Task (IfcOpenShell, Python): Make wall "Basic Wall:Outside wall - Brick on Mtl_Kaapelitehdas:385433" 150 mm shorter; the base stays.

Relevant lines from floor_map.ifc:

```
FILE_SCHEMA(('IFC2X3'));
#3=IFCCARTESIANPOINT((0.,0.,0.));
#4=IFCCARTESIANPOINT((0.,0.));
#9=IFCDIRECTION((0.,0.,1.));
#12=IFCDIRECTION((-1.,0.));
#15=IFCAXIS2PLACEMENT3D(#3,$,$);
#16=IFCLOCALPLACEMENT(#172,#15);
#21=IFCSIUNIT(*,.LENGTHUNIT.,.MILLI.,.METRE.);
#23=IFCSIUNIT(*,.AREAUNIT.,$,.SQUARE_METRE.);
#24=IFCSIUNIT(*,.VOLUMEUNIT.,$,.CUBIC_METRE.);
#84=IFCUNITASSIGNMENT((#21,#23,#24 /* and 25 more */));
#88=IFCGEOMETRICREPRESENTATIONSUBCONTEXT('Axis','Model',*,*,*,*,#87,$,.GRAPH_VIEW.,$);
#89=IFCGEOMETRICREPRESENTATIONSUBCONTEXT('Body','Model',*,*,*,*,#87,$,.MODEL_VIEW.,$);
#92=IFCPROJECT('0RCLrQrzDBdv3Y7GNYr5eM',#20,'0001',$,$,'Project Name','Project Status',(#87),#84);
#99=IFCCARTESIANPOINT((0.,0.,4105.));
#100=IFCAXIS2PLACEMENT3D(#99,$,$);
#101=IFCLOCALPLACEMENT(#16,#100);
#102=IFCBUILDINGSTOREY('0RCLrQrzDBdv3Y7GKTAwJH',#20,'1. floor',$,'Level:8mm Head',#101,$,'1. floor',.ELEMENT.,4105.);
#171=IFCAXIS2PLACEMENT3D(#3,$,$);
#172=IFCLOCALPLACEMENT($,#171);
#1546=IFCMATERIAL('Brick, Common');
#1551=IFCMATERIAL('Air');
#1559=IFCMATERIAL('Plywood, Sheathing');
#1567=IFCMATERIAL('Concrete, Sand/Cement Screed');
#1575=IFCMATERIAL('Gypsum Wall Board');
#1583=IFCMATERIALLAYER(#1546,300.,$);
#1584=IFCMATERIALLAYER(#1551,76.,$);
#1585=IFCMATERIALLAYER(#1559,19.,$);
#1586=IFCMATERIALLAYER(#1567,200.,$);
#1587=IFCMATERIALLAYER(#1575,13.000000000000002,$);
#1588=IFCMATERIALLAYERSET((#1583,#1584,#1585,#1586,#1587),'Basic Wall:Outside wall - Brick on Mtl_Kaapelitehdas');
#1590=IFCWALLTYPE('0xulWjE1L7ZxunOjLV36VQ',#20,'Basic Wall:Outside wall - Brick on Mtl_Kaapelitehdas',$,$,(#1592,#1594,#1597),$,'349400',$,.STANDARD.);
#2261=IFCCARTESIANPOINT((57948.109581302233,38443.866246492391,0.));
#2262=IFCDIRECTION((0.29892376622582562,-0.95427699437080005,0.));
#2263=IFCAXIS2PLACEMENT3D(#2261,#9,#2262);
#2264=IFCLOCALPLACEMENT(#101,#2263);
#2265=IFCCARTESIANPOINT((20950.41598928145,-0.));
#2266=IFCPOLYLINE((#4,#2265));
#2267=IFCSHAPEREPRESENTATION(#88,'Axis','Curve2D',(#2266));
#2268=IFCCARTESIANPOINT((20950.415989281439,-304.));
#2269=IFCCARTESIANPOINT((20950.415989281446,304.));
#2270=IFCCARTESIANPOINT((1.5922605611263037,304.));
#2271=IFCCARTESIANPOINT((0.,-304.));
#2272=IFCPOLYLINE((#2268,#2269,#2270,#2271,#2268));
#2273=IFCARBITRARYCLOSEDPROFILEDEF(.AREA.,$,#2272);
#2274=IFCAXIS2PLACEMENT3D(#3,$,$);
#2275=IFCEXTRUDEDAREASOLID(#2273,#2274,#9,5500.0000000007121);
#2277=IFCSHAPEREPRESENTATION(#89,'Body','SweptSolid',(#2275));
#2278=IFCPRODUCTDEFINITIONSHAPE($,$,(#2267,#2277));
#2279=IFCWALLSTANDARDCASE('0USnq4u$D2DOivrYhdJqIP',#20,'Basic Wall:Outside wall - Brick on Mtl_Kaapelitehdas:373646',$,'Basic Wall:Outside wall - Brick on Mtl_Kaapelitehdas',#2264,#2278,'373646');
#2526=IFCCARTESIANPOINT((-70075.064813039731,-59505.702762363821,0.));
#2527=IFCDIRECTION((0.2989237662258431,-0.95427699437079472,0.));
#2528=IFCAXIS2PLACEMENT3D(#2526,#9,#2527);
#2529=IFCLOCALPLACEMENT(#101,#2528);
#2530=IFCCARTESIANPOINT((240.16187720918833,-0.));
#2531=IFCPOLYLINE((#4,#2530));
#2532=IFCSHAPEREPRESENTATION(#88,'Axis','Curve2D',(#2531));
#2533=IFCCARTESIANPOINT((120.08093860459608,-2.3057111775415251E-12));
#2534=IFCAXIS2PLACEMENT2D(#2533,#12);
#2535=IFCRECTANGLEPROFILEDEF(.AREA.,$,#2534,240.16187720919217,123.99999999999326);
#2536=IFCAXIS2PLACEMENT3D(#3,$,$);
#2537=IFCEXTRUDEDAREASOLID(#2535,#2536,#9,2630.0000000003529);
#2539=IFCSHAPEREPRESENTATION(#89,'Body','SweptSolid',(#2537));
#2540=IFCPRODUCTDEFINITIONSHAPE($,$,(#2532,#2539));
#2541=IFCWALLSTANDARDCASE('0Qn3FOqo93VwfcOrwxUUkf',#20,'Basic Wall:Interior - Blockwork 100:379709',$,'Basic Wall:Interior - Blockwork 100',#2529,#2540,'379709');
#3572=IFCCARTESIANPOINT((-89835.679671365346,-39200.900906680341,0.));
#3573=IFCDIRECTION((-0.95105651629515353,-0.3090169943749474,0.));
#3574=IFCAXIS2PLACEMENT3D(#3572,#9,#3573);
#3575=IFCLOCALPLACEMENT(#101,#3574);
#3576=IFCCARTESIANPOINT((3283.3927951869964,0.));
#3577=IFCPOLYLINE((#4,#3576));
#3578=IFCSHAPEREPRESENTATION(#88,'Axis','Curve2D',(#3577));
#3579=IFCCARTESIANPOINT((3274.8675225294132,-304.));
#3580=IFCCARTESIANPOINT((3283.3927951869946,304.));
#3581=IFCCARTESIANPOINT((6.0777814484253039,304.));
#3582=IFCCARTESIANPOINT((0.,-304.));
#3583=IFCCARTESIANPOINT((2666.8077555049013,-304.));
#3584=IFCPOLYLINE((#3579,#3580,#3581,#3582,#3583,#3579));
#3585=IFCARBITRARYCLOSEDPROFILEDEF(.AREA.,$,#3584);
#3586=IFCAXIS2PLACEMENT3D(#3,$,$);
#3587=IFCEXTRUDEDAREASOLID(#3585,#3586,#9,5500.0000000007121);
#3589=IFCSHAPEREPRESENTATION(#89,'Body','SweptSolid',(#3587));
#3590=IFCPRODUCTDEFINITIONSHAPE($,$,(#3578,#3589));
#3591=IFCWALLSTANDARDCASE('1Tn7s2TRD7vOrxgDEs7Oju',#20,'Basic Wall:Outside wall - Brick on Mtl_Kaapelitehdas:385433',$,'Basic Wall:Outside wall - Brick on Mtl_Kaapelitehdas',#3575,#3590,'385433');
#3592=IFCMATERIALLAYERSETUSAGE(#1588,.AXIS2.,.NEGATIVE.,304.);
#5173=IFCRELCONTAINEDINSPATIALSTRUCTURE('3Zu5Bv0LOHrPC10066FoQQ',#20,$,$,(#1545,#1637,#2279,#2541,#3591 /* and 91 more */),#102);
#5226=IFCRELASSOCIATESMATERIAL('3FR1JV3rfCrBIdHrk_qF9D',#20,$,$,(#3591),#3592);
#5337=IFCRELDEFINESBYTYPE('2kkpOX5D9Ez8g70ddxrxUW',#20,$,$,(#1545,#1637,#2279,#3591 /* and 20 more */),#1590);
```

```python
import ifcopenshell
import ifcopenshell.geom
import ifcopenshell.util.representation
import ifcopenshell.util.shape

model = ifcopenshell.open("floor_map.ifc")
settings = ifcopenshell.geom.settings()


def volume(element):
    """Net volume in cubic metres, openings subtracted."""
    shape = ifcopenshell.geom.create_shape(settings, element)
    return ifcopenshell.util.shape.get_volume(shape.geometry)


wall = model.by_guid("1Tn7s2TRD7vOrxgDEs7Oju")
before = volume(wall)

body = ifcopenshell.util.representation.get_representation(wall, "Model", "Body")
solid = body.Items[0]
old_height = solid.Depth
solid.Depth -= 150.0
after = volume(wall)

print(f"height {old_height:g} -> {solid.Depth:g}, volume {before:.3f} -> {after:.3f} m3")

model.write("floor_map-out.ifc")
```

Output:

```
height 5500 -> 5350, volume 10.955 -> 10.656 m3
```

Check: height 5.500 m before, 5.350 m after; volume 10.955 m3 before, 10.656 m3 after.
